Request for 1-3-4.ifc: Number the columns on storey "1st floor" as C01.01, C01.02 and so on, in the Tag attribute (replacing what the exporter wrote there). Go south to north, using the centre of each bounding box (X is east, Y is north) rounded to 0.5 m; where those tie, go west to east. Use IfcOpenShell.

First a look at what the model holds.

```python
import ifcopenshell
import ifcopenshell.util.element
import ifcopenshell.util.placement

model = ifcopenshell.open("1-3-4.ifc")
print(model.schema)
storey = next(s for s in model.by_type("IfcBuildingStorey") if s.Name == "1st floor")
columns = [e for e in ifcopenshell.util.element.get_decomposition(storey) if e.is_a("IfcColumn")]
for e in sorted(columns, key=lambda e: e.id()):
    origin = ifcopenshell.util.placement.get_local_placement(e.ObjectPlacement)[:3, 3]
    print(e.id(), e.Tag, e.Name, origin.round(2) + 0.0, sep=" | ")
```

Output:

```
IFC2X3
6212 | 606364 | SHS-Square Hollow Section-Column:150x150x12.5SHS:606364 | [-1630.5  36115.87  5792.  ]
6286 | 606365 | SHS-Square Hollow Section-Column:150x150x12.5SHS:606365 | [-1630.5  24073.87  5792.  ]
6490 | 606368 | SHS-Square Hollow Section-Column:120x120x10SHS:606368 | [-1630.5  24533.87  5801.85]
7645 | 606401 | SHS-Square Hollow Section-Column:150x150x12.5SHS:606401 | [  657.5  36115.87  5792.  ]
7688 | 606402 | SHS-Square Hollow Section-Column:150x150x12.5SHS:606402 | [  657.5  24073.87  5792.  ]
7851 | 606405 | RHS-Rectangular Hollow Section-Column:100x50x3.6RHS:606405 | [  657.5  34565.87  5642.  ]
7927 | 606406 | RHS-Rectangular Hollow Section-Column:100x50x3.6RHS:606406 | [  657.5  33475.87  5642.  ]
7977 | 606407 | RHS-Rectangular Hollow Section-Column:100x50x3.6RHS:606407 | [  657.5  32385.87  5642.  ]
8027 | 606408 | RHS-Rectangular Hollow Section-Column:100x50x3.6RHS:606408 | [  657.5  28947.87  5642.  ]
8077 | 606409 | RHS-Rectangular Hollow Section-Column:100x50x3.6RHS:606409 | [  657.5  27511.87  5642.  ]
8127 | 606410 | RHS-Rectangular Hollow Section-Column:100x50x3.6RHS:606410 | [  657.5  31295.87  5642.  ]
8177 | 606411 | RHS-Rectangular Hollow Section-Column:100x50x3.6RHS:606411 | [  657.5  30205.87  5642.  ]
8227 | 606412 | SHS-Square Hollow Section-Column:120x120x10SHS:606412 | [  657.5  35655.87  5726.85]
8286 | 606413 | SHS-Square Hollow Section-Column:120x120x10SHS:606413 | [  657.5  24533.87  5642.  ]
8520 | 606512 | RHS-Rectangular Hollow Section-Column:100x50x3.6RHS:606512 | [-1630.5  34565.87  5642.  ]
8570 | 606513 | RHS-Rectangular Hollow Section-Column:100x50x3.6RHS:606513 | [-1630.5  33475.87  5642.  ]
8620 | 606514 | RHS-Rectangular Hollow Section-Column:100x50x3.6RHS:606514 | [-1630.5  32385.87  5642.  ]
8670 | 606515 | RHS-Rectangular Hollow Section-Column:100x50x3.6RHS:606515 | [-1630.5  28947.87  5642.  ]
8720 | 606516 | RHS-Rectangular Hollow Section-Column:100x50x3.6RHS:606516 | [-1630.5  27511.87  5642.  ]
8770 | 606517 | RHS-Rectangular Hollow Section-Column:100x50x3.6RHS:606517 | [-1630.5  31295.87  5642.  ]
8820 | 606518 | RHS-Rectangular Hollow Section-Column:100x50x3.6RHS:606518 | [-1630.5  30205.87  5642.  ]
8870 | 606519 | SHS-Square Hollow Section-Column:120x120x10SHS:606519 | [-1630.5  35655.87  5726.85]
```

```python
import ifcopenshell
import ifcopenshell.geom
import ifcopenshell.util.element
import ifcopenshell.util.shape

model = ifcopenshell.open("1-3-4.ifc")
settings = ifcopenshell.geom.settings()
settings.set("use-world-coords", True)


def centre(element):
    shape = ifcopenshell.geom.create_shape(settings, element)
    return ifcopenshell.util.shape.get_bbox_centroid(shape.geometry)


storey = next(s for s in model.by_type("IfcBuildingStorey") if s.Name == "1st floor")
columns = [e for e in ifcopenshell.util.element.get_decomposition(storey) if e.is_a("IfcColumn")]

# Insertion points can sit at a corner or the storey origin, so sort by the geometry (in metres).
centres = {e: centre(e) for e in columns}
columns.sort(key=lambda e: (round(centres[e][1] / 0.5), centres[e][0]))

for i, e in enumerate(columns, start=1):
    number = f"C01.{i:02d}"
    e.Tag = number
    print(e.id(), number)

model.write("1-3-4_rev.ifc")
```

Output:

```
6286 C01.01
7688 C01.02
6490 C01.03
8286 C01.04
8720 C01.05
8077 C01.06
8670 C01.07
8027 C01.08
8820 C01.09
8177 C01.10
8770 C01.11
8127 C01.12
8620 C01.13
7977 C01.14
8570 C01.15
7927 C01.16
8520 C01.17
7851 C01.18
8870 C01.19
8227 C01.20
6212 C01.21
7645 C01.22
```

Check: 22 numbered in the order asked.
